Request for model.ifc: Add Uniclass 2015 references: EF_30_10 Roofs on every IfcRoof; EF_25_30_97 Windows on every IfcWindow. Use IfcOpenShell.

First a look at what the model holds.

```python
import ifcopenshell

model = ifcopenshell.open("model.ifc")
print(model.schema)
print("classifications:", [c.Name for c in model.by_type("IfcClassification")])
for ifc_class in ("IfcDoor", "IfcRoof", "IfcStair", "IfcWall", "IfcWindow"):
    print(ifc_class, len(model.by_type(ifc_class)))
```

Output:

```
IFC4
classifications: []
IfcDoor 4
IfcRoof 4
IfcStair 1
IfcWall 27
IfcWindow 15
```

```python
import ifcopenshell
import ifcopenshell.api.classification

model = ifcopenshell.open("model.ifc")

system = ifcopenshell.api.classification.add_classification(model, classification="Uniclass 2015")

codes = {
    "IfcRoof": ("EF_30_10", "Roofs"),
    "IfcWindow": ("EF_25_30_97", "Windows"),
}
for ifc_class, (code, name) in codes.items():
    products = model.by_type(ifc_class)
    ifcopenshell.api.classification.add_reference(
        model, products=products, classification=system, identification=code, name=name
    )
    print(code, len(products))

model.write("model-out.ifc")
```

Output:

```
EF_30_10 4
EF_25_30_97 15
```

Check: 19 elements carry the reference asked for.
